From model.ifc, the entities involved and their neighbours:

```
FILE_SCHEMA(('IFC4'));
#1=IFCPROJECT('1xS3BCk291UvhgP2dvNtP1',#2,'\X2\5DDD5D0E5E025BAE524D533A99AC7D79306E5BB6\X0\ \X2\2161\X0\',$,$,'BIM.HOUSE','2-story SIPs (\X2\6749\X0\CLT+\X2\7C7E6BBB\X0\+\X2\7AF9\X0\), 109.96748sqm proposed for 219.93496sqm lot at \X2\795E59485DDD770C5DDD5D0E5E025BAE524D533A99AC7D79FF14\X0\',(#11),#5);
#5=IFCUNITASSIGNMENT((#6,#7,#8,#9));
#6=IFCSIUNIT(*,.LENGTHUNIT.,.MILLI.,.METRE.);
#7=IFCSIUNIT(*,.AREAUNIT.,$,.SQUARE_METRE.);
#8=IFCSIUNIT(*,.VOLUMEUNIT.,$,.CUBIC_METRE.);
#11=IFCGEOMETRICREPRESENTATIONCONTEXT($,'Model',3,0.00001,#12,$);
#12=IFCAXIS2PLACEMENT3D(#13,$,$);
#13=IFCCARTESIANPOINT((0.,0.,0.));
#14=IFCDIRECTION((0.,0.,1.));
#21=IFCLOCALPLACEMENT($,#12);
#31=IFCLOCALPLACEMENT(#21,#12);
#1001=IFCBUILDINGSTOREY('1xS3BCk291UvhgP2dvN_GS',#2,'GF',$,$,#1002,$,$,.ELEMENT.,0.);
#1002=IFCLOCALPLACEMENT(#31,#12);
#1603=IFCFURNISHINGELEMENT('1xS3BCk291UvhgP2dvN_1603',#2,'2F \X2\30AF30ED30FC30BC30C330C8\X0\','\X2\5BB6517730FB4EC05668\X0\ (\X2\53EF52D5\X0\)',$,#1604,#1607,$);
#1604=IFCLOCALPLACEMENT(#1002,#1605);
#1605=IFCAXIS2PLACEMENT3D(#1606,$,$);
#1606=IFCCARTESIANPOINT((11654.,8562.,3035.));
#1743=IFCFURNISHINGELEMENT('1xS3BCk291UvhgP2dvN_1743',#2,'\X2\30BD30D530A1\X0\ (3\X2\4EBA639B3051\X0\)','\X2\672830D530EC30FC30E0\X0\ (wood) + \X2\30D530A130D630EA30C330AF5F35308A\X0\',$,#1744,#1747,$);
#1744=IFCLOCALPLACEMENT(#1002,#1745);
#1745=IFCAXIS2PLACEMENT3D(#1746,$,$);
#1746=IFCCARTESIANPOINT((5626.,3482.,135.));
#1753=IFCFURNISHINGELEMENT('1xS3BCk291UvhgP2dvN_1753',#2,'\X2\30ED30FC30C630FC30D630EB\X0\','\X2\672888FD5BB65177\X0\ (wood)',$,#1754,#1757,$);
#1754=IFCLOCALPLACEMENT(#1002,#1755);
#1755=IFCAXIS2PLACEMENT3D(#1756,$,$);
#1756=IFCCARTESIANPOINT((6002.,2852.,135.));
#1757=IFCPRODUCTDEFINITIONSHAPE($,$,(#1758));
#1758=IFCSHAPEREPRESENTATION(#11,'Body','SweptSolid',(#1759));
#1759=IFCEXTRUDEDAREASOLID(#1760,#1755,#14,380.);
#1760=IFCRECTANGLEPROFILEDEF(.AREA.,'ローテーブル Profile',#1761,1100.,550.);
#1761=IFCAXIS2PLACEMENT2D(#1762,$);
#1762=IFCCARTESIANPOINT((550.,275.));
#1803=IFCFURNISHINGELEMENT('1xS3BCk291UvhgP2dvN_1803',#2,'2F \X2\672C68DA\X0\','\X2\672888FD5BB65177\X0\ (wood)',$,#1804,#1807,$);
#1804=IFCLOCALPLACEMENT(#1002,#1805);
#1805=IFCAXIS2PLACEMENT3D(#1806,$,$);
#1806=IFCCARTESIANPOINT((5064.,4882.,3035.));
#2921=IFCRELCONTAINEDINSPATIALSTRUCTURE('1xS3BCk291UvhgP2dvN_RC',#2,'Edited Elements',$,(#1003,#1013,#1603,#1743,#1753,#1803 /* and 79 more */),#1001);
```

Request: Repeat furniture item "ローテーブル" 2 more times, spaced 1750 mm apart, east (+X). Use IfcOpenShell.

```python
import numpy as np
import ifcopenshell
import ifcopenshell.api.geometry
import ifcopenshell.api.root
import ifcopenshell.util.element
import ifcopenshell.util.placement
import ifcopenshell.util.unit

model = ifcopenshell.open("model.ifc")
unit_scale = ifcopenshell.util.unit.calculate_unit_scale(model)


def reuse_history(source, copy):
    """copy_class also copies each property set's owner history, people and application; keep the originals."""
    for rel in copy.IsDefinedBy:
        if rel.is_a("IfcRelDefinesByProperties") and (history := rel.RelatingPropertyDefinition.OwnerHistory):
            rel.RelatingPropertyDefinition.OwnerHistory = source.OwnerHistory
            ifcopenshell.util.element.remove_deep2(model, history)


source = model.by_guid("1xS3BCk291UvhgP2dvN_1753")
base = ifcopenshell.util.placement.get_local_placement(source.ObjectPlacement)
step = np.array([1.0, 0.0, 0.0]) * 1.75 / unit_scale

for i in range(1, 3):
    copy = ifcopenshell.api.root.copy_class(model, product=source)
    copy.Representation = ifcopenshell.util.element.copy_deep(
        model, source.Representation, exclude=["IfcGeometricRepresentationContext", "IfcRepresentationMap"]
    )
    reuse_history(source, copy)
    matrix = base.copy()
    matrix[:3, 3] += i * step
    print("added at", matrix[:3, 3].round(3) + 0.0)
    ifcopenshell.api.geometry.edit_object_placement(model, product=copy, matrix=matrix, is_si=False)

model.write("model_v2.ifc")
```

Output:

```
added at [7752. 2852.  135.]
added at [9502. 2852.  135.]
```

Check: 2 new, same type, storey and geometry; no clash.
